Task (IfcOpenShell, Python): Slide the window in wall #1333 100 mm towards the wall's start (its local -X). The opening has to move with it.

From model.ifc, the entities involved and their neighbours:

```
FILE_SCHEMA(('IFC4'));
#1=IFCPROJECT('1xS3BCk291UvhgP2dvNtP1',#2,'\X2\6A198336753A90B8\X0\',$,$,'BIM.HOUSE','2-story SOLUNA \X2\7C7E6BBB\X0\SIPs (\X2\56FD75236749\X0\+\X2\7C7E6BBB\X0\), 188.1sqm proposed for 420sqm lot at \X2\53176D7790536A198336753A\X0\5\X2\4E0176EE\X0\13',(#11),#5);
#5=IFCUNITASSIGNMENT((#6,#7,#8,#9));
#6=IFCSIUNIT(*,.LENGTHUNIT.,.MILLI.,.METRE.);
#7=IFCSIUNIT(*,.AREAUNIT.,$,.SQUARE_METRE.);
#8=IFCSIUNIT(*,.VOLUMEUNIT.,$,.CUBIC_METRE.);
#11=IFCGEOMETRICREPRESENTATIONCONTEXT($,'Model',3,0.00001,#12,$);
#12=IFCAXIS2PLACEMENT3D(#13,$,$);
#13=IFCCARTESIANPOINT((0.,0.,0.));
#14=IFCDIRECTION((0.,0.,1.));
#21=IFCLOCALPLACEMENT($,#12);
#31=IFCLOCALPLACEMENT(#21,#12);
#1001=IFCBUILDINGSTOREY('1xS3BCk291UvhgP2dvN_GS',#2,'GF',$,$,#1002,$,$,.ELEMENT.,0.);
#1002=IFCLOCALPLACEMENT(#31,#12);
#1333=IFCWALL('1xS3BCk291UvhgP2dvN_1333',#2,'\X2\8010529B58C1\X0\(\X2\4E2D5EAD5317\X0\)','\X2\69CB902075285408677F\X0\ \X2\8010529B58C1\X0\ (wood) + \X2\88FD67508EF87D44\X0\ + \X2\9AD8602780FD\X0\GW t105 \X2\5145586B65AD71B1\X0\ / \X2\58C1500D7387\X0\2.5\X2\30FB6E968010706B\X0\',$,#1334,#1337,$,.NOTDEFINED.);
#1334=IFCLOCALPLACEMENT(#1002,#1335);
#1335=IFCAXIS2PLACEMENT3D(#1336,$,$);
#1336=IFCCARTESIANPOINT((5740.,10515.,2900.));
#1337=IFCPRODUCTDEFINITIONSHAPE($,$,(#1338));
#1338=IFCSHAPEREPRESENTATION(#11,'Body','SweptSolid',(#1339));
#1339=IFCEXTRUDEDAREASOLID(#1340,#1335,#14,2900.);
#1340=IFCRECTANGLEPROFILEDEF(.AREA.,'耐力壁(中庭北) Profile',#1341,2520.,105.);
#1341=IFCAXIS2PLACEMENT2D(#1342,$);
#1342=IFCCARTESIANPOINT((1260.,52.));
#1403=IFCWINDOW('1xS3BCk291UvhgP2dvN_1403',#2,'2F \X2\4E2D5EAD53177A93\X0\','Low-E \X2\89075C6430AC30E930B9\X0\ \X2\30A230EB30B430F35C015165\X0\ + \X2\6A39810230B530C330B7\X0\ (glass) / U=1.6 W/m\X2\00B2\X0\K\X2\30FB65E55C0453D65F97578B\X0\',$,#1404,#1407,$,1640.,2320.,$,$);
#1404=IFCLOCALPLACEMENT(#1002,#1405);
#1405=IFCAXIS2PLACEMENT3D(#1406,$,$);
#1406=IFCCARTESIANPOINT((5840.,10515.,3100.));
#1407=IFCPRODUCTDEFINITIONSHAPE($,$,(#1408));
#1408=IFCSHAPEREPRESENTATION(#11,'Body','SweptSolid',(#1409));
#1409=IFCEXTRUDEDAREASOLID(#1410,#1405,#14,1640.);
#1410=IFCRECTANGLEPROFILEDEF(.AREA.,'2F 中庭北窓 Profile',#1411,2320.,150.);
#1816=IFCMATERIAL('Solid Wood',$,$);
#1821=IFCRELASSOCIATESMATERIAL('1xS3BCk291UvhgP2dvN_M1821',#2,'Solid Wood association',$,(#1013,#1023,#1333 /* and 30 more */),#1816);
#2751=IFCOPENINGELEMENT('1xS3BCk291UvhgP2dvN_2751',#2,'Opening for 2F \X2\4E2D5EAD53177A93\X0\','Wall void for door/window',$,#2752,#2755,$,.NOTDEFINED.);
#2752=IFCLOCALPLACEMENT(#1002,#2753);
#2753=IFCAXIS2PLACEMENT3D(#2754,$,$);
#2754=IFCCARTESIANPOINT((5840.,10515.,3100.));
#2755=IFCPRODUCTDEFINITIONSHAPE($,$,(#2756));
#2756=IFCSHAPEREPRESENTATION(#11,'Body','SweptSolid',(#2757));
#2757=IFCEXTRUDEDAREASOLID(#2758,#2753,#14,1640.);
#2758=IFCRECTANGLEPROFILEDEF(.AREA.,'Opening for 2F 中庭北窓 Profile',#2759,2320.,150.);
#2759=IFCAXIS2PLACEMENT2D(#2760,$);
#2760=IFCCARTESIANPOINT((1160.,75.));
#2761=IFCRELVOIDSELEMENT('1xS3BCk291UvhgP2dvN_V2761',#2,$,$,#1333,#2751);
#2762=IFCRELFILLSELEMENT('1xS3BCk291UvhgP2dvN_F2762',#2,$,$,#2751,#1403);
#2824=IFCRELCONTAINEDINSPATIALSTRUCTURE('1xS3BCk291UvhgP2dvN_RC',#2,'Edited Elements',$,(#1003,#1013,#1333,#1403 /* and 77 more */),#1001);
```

```python
import ifcopenshell
import ifcopenshell.api.geometry
import ifcopenshell.util.placement

model = ifcopenshell.open("model.ifc")

window = model.by_guid("1xS3BCk291UvhgP2dvN_1403")
opening = window.FillsVoids[0].RelatingOpeningElement
wall = opening.VoidsElements[0].RelatingBuildingElement

wall_matrix = ifcopenshell.util.placement.get_local_placement(wall.ObjectPlacement)
shift = wall_matrix[:3, 0] * -100.0
before = ifcopenshell.util.placement.get_local_placement(window.ObjectPlacement)[:3, 3].copy()

# The window is not placed relative to its opening, so move both.
for product in (opening, window):
    matrix = ifcopenshell.util.placement.get_local_placement(product.ObjectPlacement)
    matrix[:3, 3] += shift
    ifcopenshell.api.geometry.edit_object_placement(model, product=product, matrix=matrix, is_si=False)

after = ifcopenshell.util.placement.get_local_placement(window.ObjectPlacement)[:3, 3]
print("window moved by", (after - before).round(3) + 0.0)

model.write("model_edited.ifc")
```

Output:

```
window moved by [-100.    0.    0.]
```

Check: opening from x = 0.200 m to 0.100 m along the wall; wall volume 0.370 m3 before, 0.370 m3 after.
